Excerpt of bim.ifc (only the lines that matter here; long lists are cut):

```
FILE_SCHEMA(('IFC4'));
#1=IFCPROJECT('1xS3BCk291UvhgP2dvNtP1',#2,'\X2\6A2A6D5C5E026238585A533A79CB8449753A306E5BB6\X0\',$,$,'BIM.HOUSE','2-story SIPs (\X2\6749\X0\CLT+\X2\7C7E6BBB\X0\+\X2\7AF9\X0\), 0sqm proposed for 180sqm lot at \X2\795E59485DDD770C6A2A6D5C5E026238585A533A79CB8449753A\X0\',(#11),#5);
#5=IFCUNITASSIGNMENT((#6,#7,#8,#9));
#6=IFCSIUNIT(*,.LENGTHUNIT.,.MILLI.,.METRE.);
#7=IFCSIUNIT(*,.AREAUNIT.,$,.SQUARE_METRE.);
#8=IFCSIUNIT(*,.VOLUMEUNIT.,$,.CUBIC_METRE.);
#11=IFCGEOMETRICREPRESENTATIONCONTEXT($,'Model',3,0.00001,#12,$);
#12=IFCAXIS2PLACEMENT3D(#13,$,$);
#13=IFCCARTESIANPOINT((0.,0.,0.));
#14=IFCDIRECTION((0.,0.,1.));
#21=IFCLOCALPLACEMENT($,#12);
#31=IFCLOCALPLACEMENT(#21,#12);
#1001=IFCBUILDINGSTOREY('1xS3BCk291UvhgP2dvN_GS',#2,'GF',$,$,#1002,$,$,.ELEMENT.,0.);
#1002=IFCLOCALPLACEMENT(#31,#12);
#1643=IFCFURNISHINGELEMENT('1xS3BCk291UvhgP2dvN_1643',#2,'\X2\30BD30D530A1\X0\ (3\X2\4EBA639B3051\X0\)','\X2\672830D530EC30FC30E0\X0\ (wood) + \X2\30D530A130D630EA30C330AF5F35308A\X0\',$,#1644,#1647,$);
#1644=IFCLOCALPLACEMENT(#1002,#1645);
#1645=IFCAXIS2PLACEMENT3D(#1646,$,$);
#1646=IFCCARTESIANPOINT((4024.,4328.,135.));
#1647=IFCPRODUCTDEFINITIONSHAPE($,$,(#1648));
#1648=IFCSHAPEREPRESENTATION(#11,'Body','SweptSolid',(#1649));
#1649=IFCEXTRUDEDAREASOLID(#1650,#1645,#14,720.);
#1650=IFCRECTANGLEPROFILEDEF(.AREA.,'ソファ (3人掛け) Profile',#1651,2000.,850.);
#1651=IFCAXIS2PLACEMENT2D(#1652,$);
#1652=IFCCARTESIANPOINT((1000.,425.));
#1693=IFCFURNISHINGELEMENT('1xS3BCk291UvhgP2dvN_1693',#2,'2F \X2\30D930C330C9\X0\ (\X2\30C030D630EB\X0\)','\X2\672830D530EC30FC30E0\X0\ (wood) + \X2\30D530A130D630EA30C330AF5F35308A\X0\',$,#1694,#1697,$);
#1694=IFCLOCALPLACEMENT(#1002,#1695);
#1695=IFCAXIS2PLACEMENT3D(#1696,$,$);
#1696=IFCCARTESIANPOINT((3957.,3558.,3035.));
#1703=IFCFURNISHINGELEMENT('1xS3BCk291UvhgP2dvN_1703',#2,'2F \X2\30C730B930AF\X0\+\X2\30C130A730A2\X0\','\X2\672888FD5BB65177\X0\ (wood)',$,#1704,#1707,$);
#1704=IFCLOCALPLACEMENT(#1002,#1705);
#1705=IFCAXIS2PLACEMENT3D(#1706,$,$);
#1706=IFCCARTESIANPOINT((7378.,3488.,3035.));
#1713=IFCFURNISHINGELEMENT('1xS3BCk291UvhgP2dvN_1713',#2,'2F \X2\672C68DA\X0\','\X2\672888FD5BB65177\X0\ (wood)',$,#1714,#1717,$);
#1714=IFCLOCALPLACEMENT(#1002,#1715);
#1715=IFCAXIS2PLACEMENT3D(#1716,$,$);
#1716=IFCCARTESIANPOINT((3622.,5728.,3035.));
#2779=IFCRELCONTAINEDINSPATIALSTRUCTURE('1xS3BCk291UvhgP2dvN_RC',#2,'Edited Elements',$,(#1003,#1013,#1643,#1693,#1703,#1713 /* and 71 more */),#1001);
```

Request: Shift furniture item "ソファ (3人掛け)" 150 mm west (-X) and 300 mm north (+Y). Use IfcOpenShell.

```python
import ifcopenshell
import ifcopenshell.api.geometry
import ifcopenshell.util.placement
import ifcopenshell.util.unit

model = ifcopenshell.open("bim.ifc")
unit_scale = ifcopenshell.util.unit.calculate_unit_scale(model)

item = model.by_guid("1xS3BCk291UvhgP2dvN_1643")
matrix = ifcopenshell.util.placement.get_local_placement(item.ObjectPlacement)
matrix[0, 3] -= 0.15 / unit_scale
matrix[1, 3] += 0.3 / unit_scale
ifcopenshell.api.geometry.edit_object_placement(model, product=item, matrix=matrix, is_si=False)

print(ifcopenshell.util.placement.get_local_placement(item.ObjectPlacement).round(3) + 0.0)

model.write("bim_rev.ifc")
```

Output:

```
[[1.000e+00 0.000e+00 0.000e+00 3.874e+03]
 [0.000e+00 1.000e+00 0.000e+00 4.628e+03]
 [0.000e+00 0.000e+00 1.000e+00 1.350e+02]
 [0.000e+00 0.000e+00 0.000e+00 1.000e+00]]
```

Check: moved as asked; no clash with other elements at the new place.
